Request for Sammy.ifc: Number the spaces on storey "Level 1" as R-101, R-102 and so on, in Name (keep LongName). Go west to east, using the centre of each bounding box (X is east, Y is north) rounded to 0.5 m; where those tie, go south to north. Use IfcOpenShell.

First a look at what the model holds.

```python
import ifcopenshell
import ifcopenshell.util.element
import ifcopenshell.util.placement

model = ifcopenshell.open("Sammy.ifc")
print(model.schema)
storey = next(s for s in model.by_type("IfcBuildingStorey") if s.Name == "Level 1")
spaces = [e for e in ifcopenshell.util.element.get_decomposition(storey) if e.is_a("IfcSpace")]
for e in sorted(spaces, key=lambda e: e.id()):
    origin = ifcopenshell.util.placement.get_local_placement(e.ObjectPlacement)[:3, 3]
    print(e.id(), e.Name, e.LongName, origin.round(2) + 0.0, sep=" | ")
```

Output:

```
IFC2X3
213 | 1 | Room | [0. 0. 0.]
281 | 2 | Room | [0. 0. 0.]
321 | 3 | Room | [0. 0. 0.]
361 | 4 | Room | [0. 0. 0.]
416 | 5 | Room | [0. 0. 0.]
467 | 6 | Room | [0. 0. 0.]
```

```python
import ifcopenshell
import ifcopenshell.geom
import ifcopenshell.util.element
import ifcopenshell.util.shape

model = ifcopenshell.open("Sammy.ifc")
settings = ifcopenshell.geom.settings()
settings.set("use-world-coords", True)


def centre(element):
    shape = ifcopenshell.geom.create_shape(settings, element)
    return ifcopenshell.util.shape.get_bbox_centroid(shape.geometry)


storey = next(s for s in model.by_type("IfcBuildingStorey") if s.Name == "Level 1")
spaces = [e for e in ifcopenshell.util.element.get_decomposition(storey) if e.is_a("IfcSpace")]

# Insertion points can sit at a corner or the storey origin, so sort by the geometry (in metres).
centres = {e: centre(e) for e in spaces}
spaces.sort(key=lambda e: (round(centres[e][0] / 0.5), centres[e][1]))

for i, e in enumerate(spaces, start=1):
    number = f"R-1{i:02d}"
    e.Name = number
    print(e.id(), number)

model.write("Sammy-out.ifc")
```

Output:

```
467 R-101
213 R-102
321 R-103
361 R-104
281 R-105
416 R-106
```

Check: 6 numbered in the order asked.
